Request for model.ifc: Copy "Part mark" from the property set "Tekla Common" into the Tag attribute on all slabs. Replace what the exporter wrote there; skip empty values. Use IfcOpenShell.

First a look at what the model holds.

```python
import ifcopenshell
import ifcopenshell.util.element

model = ifcopenshell.open("model.ifc")
print(model.schema)
slabs = model.by_type("IfcSlab")
print(len(slabs), "slabs")
for e in slabs[:8]:
    source = ifcopenshell.util.element.get_pset(e, "Tekla Common", "Part mark")
    target = e.Tag
    print(e.id(), repr(source), repr(target), sep=" | ")
```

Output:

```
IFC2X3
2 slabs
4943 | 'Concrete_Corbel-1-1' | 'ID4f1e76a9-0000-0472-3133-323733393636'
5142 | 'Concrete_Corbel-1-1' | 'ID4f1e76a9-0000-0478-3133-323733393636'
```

```python
import ifcopenshell
import ifcopenshell.util.element

model = ifcopenshell.open("model.ifc")

count = 0
for e in model.by_type("IfcSlab"):
    value = ifcopenshell.util.element.get_pset(e, "Tekla Common", "Part mark")
    current = e.Tag
    if not value or not value.strip() or current == value:
        continue
    e.Tag = value
    count += 1

print(count, "slabs updated")

model.write("model_updated.ifc")
```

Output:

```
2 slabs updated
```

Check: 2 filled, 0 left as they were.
